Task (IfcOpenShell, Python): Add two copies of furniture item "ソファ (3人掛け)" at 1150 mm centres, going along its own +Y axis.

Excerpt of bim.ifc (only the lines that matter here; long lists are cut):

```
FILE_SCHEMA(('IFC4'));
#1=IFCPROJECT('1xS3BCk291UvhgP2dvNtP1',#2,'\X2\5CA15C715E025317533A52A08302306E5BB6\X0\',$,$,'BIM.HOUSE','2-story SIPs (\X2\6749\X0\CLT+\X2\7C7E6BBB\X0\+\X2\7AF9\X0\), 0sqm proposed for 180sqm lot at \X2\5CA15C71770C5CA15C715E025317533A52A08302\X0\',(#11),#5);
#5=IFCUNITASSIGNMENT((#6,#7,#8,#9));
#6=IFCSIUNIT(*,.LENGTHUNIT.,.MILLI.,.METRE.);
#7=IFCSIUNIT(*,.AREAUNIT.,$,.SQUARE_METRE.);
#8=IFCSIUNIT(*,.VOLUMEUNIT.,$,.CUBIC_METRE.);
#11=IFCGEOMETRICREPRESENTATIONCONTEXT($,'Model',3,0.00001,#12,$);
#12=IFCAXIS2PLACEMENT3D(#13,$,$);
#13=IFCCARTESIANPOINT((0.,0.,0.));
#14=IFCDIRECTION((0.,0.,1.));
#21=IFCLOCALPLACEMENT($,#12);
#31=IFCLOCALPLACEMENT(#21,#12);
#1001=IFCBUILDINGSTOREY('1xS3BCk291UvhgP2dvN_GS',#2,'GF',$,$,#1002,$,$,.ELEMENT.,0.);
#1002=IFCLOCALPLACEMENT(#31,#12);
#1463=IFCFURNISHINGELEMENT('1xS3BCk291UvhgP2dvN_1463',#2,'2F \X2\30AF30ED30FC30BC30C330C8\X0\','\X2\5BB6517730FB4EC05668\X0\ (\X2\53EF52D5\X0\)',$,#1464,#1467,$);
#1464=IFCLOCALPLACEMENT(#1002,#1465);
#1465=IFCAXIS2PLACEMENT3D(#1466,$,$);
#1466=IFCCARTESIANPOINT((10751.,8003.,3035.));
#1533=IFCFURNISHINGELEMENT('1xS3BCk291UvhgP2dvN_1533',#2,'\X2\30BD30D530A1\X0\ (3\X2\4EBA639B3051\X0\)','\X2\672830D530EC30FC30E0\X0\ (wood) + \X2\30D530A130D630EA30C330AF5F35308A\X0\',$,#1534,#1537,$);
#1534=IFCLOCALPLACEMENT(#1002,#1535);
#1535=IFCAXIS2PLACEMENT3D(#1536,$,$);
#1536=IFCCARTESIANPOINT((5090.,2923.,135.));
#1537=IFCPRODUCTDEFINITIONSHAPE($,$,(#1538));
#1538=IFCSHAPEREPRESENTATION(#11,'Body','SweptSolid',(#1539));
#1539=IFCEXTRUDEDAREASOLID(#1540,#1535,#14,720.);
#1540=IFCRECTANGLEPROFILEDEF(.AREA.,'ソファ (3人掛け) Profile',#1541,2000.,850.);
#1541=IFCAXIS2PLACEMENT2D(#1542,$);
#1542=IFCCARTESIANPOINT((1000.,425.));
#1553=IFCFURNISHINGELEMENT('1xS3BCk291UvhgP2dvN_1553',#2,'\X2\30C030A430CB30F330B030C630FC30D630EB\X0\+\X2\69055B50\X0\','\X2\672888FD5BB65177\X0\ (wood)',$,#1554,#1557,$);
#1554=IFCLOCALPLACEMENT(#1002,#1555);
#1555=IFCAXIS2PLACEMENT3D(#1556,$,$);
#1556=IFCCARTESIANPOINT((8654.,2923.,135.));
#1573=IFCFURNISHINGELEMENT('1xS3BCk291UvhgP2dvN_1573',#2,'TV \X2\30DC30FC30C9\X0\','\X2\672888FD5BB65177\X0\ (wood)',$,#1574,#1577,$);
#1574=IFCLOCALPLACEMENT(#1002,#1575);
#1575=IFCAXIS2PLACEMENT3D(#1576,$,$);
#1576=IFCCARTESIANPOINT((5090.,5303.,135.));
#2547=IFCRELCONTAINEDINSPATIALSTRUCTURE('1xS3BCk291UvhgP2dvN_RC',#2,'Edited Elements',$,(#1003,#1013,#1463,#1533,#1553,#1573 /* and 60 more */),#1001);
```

```python
import ifcopenshell
import ifcopenshell.api.geometry
import ifcopenshell.api.root
import ifcopenshell.util.element
import ifcopenshell.util.placement
import ifcopenshell.util.unit

model = ifcopenshell.open("bim.ifc")
unit_scale = ifcopenshell.util.unit.calculate_unit_scale(model)


def reuse_history(source, copy):
    """copy_class also copies each property set's owner history, people and application; keep the originals."""
    for rel in copy.IsDefinedBy:
        if rel.is_a("IfcRelDefinesByProperties") and (history := rel.RelatingPropertyDefinition.OwnerHistory):
            rel.RelatingPropertyDefinition.OwnerHistory = source.OwnerHistory
            ifcopenshell.util.element.remove_deep2(model, history)


source = model.by_id(1533)
base = ifcopenshell.util.placement.get_local_placement(source.ObjectPlacement)
step = base[:3, 1] * 1.15 / unit_scale

for i in range(1, 3):
    copy = ifcopenshell.api.root.copy_class(model, product=source)
    copy.Representation = ifcopenshell.util.element.copy_deep(
        model, source.Representation, exclude=["IfcGeometricRepresentationContext", "IfcRepresentationMap"]
    )
    reuse_history(source, copy)
    matrix = base.copy()
    matrix[:3, 3] += i * step
    print("added at", matrix[:3, 3].round(3) + 0.0)
    ifcopenshell.api.geometry.edit_object_placement(model, product=copy, matrix=matrix, is_si=False)

model.write("bim_edited.ifc")
```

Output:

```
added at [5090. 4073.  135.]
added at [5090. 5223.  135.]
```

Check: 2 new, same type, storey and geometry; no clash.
